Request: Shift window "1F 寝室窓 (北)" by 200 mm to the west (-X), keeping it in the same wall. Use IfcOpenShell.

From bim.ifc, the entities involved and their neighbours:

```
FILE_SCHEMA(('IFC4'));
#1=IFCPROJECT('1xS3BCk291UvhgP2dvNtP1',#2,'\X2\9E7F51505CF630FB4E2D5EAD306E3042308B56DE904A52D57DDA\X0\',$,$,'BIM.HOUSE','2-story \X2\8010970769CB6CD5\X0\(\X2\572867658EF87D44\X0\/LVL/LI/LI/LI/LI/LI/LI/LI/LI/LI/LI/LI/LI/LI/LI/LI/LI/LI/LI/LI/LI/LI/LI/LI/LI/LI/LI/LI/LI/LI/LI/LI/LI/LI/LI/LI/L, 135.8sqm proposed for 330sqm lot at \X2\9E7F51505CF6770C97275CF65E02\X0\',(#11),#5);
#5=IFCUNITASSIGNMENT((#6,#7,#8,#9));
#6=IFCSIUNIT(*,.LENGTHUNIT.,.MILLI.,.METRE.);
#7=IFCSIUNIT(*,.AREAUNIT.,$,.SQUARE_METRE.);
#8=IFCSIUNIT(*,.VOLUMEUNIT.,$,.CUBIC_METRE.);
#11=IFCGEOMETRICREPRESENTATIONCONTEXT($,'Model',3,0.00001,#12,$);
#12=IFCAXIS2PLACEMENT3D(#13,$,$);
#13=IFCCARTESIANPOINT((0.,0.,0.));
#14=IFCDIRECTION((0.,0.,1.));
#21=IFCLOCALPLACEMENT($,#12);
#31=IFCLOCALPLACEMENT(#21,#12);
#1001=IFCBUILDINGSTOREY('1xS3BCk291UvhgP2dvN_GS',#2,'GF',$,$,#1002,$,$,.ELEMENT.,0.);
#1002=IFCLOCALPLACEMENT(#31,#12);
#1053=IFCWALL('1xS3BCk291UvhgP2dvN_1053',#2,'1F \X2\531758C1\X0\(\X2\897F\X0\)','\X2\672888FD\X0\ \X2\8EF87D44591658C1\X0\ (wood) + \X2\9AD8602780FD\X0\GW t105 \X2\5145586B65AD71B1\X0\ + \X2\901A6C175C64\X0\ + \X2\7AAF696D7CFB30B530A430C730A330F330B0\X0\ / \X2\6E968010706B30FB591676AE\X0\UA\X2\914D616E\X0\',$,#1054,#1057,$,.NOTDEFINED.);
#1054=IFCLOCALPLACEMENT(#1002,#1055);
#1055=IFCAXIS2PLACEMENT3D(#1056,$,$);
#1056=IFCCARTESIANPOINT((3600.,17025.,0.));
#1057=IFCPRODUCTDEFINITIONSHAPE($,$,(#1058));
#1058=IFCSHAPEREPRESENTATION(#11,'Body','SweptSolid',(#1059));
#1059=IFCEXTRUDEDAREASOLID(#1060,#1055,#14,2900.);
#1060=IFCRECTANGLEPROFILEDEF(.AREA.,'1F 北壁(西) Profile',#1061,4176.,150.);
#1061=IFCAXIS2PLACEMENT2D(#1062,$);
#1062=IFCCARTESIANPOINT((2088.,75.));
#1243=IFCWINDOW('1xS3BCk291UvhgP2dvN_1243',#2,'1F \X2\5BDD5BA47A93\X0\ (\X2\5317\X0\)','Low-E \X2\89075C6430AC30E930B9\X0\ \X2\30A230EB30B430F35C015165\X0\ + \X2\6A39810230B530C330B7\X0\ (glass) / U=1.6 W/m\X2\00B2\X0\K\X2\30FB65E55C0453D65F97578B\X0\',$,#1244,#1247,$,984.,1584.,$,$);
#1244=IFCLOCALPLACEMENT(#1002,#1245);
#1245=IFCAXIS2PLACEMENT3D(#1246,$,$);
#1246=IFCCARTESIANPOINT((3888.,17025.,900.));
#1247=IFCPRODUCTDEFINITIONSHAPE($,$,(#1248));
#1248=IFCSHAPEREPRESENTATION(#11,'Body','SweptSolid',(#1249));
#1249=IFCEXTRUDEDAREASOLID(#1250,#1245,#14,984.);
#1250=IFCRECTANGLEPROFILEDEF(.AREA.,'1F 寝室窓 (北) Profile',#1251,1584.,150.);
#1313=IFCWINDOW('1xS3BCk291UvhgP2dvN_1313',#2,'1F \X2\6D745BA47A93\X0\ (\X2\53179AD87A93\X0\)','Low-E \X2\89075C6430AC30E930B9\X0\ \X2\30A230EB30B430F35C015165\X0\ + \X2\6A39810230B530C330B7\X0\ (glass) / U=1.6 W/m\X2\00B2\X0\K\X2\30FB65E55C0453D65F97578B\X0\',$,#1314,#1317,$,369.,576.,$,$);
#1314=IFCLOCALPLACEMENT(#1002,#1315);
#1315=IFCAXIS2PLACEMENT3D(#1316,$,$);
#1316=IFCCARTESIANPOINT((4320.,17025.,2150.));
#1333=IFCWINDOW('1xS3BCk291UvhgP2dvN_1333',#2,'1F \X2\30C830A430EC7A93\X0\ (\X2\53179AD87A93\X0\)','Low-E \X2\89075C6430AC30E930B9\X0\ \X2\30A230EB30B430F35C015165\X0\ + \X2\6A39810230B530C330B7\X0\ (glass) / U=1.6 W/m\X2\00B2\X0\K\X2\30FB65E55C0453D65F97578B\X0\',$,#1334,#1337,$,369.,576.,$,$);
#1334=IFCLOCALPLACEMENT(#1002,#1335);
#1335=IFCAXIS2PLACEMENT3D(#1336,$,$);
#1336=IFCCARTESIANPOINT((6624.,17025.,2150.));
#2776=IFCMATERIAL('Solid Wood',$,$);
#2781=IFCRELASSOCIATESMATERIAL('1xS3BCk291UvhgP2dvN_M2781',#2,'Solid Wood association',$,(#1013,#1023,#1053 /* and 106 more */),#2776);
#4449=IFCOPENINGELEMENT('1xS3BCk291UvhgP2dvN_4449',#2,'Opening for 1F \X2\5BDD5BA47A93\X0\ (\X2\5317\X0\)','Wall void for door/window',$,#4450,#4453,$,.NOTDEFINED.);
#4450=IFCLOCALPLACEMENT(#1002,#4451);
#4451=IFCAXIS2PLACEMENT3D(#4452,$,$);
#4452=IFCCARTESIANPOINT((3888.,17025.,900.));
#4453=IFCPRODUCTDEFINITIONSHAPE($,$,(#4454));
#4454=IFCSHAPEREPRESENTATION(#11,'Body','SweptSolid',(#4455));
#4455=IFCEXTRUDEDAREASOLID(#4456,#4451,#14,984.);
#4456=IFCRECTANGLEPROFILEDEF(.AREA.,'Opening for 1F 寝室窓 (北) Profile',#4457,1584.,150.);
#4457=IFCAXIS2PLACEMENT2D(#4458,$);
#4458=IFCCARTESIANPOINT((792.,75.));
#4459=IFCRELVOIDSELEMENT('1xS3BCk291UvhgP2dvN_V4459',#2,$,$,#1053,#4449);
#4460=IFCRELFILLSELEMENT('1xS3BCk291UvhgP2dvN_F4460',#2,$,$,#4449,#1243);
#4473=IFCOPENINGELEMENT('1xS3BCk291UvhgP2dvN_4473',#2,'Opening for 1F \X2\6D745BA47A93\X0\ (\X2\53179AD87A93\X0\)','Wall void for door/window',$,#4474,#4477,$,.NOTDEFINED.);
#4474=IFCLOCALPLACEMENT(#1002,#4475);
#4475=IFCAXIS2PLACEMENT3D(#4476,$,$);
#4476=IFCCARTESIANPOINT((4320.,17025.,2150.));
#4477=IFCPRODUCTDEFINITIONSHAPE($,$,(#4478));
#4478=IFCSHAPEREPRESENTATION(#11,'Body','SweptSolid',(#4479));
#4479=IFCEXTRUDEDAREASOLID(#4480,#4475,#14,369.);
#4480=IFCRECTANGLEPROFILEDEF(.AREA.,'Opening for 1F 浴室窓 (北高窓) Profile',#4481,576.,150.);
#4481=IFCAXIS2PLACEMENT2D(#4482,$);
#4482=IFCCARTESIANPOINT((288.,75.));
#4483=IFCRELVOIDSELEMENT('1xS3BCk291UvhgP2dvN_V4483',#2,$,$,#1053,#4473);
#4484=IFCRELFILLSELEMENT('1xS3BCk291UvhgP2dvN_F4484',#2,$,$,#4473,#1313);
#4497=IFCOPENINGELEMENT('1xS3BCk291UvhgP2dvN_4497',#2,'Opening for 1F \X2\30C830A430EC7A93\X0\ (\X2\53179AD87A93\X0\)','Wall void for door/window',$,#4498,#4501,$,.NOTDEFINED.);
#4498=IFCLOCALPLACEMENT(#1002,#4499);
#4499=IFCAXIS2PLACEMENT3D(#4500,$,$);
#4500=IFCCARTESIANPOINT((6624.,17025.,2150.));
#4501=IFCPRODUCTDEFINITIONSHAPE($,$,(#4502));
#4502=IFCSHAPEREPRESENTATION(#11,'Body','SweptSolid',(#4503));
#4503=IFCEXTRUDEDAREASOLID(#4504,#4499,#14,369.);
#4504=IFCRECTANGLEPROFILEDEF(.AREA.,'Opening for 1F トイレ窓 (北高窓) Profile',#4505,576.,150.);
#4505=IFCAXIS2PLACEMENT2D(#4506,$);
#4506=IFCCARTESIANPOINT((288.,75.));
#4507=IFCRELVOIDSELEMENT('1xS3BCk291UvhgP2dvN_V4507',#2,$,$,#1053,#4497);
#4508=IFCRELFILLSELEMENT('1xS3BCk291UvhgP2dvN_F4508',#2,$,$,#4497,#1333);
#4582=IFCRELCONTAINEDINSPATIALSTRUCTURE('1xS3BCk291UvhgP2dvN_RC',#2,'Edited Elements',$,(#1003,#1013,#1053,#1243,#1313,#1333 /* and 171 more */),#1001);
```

```python
import ifcopenshell
import ifcopenshell.api.geometry
import ifcopenshell.util.placement

model = ifcopenshell.open("bim.ifc")

window = model.by_guid("1xS3BCk291UvhgP2dvN_1243")
opening = window.FillsVoids[0].RelatingOpeningElement
wall = opening.VoidsElements[0].RelatingBuildingElement

wall_matrix = ifcopenshell.util.placement.get_local_placement(wall.ObjectPlacement)
shift = wall_matrix[:3, 0] * -200.0
before = ifcopenshell.util.placement.get_local_placement(window.ObjectPlacement)[:3, 3].copy()

# The window is not placed relative to its opening, so move both.
for product in (opening, window):
    matrix = ifcopenshell.util.placement.get_local_placement(product.ObjectPlacement)
    matrix[:3, 3] += shift
    ifcopenshell.api.geometry.edit_object_placement(model, product=product, matrix=matrix, is_si=False)

after = ifcopenshell.util.placement.get_local_placement(window.ObjectPlacement)[:3, 3]
print("window moved by", (after - before).round(3) + 0.0)

model.write("bim_edited.ifc")
```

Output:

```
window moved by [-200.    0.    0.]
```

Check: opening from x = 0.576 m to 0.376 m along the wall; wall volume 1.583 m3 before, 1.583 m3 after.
